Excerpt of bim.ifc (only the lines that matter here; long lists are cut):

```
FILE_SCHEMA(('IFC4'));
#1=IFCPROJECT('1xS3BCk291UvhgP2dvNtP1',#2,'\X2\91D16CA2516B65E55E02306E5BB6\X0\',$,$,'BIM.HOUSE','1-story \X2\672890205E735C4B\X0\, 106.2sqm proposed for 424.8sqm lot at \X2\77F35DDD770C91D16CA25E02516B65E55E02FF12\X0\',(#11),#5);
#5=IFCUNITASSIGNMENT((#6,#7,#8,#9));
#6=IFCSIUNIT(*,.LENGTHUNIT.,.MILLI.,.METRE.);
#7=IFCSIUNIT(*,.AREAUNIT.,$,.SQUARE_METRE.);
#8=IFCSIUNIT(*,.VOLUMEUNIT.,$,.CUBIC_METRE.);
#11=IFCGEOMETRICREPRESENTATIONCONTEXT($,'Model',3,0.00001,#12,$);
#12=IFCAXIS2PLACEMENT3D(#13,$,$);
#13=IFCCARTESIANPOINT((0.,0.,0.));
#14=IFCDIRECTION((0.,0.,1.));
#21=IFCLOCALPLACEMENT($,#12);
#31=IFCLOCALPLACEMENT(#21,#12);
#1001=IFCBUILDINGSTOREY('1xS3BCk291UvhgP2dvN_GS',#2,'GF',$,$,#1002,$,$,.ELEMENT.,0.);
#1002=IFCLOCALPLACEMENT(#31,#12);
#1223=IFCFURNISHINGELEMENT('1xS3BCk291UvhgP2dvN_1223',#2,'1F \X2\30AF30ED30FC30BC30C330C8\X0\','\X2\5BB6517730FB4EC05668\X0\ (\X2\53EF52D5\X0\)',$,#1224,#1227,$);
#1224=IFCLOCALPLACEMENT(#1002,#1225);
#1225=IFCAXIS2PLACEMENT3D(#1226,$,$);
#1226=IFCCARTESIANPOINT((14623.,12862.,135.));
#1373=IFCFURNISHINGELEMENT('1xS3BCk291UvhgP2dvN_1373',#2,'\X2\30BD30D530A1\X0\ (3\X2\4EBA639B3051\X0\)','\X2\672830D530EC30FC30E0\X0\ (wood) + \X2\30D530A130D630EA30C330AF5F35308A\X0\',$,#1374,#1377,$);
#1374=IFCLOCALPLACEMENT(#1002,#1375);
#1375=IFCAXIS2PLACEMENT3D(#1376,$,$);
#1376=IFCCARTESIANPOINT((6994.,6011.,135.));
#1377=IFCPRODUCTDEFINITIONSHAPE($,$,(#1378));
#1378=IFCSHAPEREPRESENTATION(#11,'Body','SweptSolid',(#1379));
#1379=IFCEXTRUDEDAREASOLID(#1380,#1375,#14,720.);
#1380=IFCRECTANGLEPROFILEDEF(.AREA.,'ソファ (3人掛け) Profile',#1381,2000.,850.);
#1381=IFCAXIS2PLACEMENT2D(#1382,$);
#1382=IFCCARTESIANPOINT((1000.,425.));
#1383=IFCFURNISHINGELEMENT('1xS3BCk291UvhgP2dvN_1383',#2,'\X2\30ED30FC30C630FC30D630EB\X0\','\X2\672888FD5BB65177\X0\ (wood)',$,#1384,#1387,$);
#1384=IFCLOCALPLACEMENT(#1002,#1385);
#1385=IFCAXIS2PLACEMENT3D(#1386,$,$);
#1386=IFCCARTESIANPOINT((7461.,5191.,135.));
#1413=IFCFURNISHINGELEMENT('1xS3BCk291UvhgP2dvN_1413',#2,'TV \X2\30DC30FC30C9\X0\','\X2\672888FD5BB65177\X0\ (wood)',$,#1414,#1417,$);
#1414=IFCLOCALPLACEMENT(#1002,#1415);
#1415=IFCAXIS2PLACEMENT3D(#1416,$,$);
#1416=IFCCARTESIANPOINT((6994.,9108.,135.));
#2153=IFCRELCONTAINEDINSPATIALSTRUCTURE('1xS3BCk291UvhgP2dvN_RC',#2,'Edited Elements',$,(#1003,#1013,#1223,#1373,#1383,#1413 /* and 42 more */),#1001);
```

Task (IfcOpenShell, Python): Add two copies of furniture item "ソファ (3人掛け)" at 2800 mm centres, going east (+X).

```python
import numpy as np
import ifcopenshell
import ifcopenshell.api.geometry
import ifcopenshell.api.root
import ifcopenshell.util.element
import ifcopenshell.util.placement
import ifcopenshell.util.unit

model = ifcopenshell.open("bim.ifc")
unit_scale = ifcopenshell.util.unit.calculate_unit_scale(model)


def reuse_history(source, copy):
    """copy_class also copies each property set's owner history, people and application; keep the originals."""
    for rel in copy.IsDefinedBy:
        if rel.is_a("IfcRelDefinesByProperties") and (history := rel.RelatingPropertyDefinition.OwnerHistory):
            rel.RelatingPropertyDefinition.OwnerHistory = source.OwnerHistory
            ifcopenshell.util.element.remove_deep2(model, history)


source = model.by_id(1373)
base = ifcopenshell.util.placement.get_local_placement(source.ObjectPlacement)
step = np.array([1.0, 0.0, 0.0]) * 2.8 / unit_scale

for i in range(1, 3):
    copy = ifcopenshell.api.root.copy_class(model, product=source)
    copy.Representation = ifcopenshell.util.element.copy_deep(
        model, source.Representation, exclude=["IfcGeometricRepresentationContext", "IfcRepresentationMap"]
    )
    reuse_history(source, copy)
    matrix = base.copy()
    matrix[:3, 3] += i * step
    print("added at", matrix[:3, 3].round(3) + 0.0)
    ifcopenshell.api.geometry.edit_object_placement(model, product=copy, matrix=matrix, is_si=False)

model.write("bim_updated.ifc")
```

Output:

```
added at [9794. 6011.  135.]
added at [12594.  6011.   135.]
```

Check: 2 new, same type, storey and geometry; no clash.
